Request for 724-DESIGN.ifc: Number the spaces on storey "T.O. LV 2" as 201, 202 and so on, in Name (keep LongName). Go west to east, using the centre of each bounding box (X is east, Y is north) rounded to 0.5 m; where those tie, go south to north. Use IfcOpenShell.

First a look at what the model holds.

```python
import ifcopenshell
import ifcopenshell.util.element
import ifcopenshell.util.placement

model = ifcopenshell.open("724-DESIGN.ifc")
print(model.schema)
storey = next(s for s in model.by_type("IfcBuildingStorey") if s.Name == "T.O. LV 2")
spaces = [e for e in ifcopenshell.util.element.get_decomposition(storey) if e.is_a("IfcSpace")]
for e in sorted(spaces, key=lambda e: e.id()):
    origin = ifcopenshell.util.placement.get_local_placement(e.ObjectPlacement)[:3, 3]
    print(e.id(), e.Name, e.LongName, origin.round(2) + 0.0, sep=" | ")
```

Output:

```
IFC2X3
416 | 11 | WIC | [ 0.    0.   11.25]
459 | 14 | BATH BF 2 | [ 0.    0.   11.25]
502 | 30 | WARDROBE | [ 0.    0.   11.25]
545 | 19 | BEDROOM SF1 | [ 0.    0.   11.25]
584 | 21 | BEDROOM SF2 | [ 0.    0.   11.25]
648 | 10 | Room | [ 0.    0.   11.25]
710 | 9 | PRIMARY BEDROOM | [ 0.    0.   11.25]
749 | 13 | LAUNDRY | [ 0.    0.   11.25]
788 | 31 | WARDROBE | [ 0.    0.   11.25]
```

```python
import ifcopenshell
import ifcopenshell.geom
import ifcopenshell.util.element
import ifcopenshell.util.shape

model = ifcopenshell.open("724-DESIGN.ifc")
settings = ifcopenshell.geom.settings()
settings.set("use-world-coords", True)


def centre(element):
    shape = ifcopenshell.geom.create_shape(settings, element)
    return ifcopenshell.util.shape.get_bbox_centroid(shape.geometry)


storey = next(s for s in model.by_type("IfcBuildingStorey") if s.Name == "T.O. LV 2")
spaces = [e for e in ifcopenshell.util.element.get_decomposition(storey) if e.is_a("IfcSpace")]

# Insertion points can sit at a corner or the storey origin, so sort by the geometry (in metres).
centres = {e: centre(e) for e in spaces}
spaces.sort(key=lambda e: (round(centres[e][0] / 0.5), centres[e][1]))

for i, e in enumerate(spaces, start=1):
    number = f"2{i:02d}"
    e.Name = number
    print(e.id(), number)

model.write("724-DESIGN_updated.ifc")
```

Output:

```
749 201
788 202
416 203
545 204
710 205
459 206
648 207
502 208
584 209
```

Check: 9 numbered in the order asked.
